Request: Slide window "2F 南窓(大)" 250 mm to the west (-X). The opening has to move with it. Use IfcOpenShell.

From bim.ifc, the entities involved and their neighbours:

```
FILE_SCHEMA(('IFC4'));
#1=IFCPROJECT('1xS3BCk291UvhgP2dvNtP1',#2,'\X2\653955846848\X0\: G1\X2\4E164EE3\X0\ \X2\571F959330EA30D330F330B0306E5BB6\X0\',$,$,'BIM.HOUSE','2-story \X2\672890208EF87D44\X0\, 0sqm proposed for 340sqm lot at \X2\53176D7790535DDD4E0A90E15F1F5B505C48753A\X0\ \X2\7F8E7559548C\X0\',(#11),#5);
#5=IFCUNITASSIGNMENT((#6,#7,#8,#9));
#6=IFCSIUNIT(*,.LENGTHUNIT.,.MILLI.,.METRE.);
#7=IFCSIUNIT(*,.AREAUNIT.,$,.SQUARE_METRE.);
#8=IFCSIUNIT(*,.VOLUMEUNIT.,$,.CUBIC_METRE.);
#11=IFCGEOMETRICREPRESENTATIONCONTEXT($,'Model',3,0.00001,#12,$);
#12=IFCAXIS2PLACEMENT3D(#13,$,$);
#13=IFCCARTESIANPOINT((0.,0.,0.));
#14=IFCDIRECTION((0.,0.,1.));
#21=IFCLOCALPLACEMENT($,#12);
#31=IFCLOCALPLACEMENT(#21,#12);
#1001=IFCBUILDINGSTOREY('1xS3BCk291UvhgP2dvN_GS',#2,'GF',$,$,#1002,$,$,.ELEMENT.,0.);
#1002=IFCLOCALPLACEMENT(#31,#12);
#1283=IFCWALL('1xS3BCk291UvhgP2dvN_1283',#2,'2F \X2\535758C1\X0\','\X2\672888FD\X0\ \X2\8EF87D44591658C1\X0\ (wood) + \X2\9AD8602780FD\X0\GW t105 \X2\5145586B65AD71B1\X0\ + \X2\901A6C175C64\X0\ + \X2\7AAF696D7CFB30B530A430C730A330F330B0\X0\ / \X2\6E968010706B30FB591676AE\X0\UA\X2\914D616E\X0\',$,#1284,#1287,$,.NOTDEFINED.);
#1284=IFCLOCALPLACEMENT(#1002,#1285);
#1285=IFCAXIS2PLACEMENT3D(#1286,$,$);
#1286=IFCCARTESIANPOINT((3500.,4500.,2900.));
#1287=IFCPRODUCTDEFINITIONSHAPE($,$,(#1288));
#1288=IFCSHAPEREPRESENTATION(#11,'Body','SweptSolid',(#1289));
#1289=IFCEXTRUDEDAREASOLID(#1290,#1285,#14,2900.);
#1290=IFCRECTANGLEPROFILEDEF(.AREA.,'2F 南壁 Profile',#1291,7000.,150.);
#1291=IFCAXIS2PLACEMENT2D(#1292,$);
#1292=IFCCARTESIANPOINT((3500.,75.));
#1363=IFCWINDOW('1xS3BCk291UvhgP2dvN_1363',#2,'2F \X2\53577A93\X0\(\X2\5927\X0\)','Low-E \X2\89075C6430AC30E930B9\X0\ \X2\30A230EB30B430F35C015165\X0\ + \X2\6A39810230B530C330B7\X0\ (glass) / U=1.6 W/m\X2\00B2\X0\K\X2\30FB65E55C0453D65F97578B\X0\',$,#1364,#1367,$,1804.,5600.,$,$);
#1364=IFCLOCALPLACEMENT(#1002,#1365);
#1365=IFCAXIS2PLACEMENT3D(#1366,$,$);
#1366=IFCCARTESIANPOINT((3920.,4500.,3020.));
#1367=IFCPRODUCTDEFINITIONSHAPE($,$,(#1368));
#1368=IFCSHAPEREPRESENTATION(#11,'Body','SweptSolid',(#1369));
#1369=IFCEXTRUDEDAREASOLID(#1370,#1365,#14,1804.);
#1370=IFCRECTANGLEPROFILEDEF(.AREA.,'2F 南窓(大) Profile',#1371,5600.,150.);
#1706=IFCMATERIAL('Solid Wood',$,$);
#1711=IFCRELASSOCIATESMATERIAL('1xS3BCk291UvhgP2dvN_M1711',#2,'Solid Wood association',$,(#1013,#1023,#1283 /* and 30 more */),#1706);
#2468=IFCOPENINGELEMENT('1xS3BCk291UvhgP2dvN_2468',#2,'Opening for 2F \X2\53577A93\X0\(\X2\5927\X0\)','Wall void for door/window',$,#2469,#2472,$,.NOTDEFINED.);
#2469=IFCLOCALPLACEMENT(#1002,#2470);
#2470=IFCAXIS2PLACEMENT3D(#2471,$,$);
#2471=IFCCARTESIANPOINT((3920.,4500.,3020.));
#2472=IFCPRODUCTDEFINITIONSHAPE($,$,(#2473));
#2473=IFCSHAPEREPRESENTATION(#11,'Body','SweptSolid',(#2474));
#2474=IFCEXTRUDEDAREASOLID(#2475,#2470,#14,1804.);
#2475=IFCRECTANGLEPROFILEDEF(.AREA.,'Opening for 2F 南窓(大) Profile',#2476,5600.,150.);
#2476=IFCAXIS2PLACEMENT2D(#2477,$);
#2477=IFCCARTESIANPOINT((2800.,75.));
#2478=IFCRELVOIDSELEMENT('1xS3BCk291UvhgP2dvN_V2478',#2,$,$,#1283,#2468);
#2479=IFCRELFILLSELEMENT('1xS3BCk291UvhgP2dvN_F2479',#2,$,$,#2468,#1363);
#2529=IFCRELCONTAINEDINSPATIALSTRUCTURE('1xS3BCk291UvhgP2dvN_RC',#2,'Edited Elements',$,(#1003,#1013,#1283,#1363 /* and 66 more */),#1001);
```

```python
import ifcopenshell
import ifcopenshell.api.geometry
import ifcopenshell.util.placement

model = ifcopenshell.open("bim.ifc")

window = model.by_id(1363)
opening = window.FillsVoids[0].RelatingOpeningElement
wall = opening.VoidsElements[0].RelatingBuildingElement

wall_matrix = ifcopenshell.util.placement.get_local_placement(wall.ObjectPlacement)
shift = wall_matrix[:3, 0] * -250.0
before = ifcopenshell.util.placement.get_local_placement(window.ObjectPlacement)[:3, 3].copy()

# The window is not placed relative to its opening, so move both.
for product in (opening, window):
    matrix = ifcopenshell.util.placement.get_local_placement(product.ObjectPlacement)
    matrix[:3, 3] += shift
    ifcopenshell.api.geometry.edit_object_placement(model, product=product, matrix=matrix, is_si=False)

after = ifcopenshell.util.placement.get_local_placement(window.ObjectPlacement)[:3, 3]
print("window moved by", (after - before).round(3) + 0.0)

model.write("bim_rev.ifc")
```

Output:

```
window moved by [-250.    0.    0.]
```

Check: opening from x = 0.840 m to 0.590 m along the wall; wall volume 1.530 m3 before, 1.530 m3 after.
